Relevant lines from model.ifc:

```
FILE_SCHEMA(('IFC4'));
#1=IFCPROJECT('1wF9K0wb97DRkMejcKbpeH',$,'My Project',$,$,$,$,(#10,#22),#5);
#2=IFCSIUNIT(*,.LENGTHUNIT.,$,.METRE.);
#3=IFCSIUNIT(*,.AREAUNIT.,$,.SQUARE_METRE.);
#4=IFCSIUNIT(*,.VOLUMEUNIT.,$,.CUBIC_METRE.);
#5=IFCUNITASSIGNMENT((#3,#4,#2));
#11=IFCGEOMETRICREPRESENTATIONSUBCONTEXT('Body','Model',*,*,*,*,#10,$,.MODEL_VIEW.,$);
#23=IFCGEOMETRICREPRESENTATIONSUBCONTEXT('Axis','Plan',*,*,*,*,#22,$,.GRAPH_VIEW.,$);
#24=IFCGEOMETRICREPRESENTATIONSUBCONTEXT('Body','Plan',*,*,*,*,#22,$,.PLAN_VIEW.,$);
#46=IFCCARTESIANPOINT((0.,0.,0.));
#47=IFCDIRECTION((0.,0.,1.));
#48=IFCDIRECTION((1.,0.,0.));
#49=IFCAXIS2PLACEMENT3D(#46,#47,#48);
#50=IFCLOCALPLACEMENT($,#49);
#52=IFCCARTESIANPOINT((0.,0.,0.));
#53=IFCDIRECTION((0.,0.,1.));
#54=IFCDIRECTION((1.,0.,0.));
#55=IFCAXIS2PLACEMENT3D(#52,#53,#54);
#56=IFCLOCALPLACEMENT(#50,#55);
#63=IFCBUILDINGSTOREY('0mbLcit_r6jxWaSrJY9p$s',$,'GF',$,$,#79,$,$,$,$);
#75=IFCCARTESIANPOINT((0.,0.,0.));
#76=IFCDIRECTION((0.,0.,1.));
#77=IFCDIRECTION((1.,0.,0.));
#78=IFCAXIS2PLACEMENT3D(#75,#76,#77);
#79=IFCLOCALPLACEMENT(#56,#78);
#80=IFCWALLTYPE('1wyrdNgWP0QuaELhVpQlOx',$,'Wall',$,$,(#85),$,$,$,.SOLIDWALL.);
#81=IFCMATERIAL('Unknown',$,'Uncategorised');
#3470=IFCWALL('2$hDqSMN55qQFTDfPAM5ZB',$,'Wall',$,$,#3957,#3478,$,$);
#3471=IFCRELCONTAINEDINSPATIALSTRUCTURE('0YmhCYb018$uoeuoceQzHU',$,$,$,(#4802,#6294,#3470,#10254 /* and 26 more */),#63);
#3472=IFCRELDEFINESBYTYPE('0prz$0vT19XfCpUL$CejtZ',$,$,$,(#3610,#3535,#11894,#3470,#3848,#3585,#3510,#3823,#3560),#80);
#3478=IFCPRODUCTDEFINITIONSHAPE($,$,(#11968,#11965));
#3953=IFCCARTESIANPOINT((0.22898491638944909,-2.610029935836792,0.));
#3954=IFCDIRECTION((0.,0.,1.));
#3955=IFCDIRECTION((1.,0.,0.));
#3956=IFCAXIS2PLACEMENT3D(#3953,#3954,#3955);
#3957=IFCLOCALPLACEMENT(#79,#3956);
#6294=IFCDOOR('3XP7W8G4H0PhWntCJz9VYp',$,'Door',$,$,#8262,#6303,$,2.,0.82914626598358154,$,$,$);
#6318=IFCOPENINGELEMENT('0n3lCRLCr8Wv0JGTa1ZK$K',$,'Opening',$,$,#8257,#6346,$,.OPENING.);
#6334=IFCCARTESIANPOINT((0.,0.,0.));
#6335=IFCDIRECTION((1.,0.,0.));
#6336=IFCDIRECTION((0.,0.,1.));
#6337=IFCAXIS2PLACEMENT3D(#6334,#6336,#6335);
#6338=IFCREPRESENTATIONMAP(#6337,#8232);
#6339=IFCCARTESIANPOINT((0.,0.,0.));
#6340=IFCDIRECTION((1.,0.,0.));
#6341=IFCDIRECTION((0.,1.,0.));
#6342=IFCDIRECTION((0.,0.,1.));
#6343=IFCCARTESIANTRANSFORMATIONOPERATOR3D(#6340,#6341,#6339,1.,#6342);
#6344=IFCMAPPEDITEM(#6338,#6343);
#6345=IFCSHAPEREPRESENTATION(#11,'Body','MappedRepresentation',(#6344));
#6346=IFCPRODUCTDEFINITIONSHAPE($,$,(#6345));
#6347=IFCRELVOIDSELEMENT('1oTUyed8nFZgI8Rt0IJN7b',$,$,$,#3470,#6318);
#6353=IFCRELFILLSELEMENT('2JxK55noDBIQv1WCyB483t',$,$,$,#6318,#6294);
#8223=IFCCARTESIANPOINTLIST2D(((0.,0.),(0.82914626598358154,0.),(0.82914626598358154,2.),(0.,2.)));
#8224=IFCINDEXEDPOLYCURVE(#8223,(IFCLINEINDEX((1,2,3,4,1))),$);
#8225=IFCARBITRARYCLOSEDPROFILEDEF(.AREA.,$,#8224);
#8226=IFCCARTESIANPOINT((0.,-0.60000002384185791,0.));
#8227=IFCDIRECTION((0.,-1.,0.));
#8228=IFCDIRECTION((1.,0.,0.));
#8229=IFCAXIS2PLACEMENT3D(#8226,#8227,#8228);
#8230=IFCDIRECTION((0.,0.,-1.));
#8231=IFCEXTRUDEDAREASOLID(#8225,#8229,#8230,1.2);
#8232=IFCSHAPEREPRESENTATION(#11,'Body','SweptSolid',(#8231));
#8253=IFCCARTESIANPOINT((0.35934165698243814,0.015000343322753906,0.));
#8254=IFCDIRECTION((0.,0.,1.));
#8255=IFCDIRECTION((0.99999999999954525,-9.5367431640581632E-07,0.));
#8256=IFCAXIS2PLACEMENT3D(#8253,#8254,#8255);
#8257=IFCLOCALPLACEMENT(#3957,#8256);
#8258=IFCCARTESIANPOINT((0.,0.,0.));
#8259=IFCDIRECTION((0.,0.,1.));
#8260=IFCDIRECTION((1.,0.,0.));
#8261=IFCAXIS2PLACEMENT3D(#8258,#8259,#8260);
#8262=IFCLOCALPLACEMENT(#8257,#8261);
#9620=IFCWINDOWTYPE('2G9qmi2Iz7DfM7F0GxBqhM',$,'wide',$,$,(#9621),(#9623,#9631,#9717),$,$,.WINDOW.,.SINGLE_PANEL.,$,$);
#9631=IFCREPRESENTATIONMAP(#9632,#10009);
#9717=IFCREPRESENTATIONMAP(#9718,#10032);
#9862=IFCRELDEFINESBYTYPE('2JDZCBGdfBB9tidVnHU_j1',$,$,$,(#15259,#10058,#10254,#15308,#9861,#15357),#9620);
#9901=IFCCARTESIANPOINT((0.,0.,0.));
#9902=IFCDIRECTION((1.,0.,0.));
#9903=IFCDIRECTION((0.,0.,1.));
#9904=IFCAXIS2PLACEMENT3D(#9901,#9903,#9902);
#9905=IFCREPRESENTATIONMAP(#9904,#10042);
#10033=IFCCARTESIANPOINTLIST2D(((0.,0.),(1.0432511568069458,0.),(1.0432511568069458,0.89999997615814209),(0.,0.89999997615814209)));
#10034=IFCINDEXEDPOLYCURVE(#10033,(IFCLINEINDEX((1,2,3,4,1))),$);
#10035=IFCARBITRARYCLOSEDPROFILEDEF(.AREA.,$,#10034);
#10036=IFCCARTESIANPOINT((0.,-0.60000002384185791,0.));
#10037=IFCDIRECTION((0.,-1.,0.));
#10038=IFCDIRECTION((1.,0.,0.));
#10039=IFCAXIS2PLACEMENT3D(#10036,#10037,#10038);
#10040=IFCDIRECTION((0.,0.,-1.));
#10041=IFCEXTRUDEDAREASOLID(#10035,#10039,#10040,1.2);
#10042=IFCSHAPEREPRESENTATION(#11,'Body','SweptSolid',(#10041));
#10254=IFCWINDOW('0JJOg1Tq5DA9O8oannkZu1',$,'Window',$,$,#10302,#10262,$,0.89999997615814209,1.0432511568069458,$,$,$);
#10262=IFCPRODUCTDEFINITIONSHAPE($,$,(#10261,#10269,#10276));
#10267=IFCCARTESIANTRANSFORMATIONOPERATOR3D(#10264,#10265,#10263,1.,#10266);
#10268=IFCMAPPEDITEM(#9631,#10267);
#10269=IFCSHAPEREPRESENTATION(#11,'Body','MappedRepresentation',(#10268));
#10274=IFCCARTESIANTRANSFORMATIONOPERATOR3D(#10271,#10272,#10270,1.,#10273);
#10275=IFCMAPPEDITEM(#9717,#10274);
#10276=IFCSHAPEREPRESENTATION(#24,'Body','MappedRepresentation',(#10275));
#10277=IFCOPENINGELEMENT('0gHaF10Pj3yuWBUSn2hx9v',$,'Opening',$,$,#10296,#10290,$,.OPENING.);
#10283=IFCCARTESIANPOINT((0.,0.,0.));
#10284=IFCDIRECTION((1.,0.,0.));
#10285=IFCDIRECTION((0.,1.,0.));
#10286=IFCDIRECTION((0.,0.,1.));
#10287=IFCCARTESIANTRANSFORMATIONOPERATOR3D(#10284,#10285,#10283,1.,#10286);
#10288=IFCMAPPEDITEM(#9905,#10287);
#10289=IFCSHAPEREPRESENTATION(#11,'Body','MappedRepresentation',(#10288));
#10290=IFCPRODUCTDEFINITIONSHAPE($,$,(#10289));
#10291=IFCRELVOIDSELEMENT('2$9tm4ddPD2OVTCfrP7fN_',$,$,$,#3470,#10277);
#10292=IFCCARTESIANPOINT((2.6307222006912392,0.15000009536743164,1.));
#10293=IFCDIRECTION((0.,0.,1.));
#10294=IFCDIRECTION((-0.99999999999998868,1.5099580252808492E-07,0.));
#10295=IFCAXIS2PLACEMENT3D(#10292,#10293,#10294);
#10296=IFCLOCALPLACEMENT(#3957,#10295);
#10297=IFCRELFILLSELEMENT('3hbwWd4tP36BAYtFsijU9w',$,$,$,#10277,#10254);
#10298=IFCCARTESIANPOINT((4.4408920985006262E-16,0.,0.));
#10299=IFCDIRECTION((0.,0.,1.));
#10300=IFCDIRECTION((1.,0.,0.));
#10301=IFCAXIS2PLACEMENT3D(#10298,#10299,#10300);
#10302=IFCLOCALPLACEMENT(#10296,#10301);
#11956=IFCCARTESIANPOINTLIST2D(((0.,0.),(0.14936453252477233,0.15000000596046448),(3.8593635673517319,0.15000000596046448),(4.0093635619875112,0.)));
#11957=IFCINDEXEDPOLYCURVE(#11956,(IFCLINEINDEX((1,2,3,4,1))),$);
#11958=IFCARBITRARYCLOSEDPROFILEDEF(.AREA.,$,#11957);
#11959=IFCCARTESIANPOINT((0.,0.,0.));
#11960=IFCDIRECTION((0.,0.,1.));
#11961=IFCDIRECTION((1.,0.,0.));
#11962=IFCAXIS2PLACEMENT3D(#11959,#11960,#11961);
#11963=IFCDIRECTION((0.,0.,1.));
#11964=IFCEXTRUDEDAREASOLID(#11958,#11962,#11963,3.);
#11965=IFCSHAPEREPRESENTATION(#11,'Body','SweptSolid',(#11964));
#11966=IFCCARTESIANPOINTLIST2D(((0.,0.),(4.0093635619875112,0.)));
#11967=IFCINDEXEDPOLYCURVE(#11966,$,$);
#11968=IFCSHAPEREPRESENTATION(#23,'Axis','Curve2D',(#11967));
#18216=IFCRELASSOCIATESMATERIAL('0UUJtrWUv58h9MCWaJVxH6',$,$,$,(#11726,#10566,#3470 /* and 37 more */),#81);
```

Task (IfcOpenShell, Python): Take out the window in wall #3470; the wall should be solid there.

```python
import ifcopenshell
import ifcopenshell.api.feature
import ifcopenshell.api.root
import ifcopenshell.geom
import ifcopenshell.util.shape

model = ifcopenshell.open("model.ifc")
settings = ifcopenshell.geom.settings()


def volume(element):
    """Net volume in cubic metres, openings subtracted."""
    shape = ifcopenshell.geom.create_shape(settings, element)
    return ifcopenshell.util.shape.get_volume(shape.geometry)


window = model.by_guid("0JJOg1Tq5DA9O8oannkZu1")
opening = window.FillsVoids[0].RelatingOpeningElement
wall = opening.VoidsElements[0].RelatingBuildingElement
before = volume(wall)

ifcopenshell.api.root.remove_product(model, product=window)
ifcopenshell.api.feature.remove_feature(model, feature=opening)

after = volume(wall)

print(f"wall volume {before:.3f} -> {after:.3f} m3")

model.write("model_edited.ifc")
```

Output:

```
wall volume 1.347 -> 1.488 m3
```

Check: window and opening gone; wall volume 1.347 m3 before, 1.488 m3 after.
